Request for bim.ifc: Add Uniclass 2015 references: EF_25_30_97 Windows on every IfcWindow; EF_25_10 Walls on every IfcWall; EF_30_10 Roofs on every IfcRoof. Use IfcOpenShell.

First a look at what the model holds.

```python
import ifcopenshell

model = ifcopenshell.open("bim.ifc")
print(model.schema)
print("classifications:", [c.Name for c in model.by_type("IfcClassification")])
for ifc_class in ("IfcDoor", "IfcRoof", "IfcStair", "IfcWall", "IfcWindow"):
    print(ifc_class, len(model.by_type(ifc_class)))
```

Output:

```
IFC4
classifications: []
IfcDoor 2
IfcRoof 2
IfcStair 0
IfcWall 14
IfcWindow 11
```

```python
import ifcopenshell
import ifcopenshell.api.classification

model = ifcopenshell.open("bim.ifc")

system = ifcopenshell.api.classification.add_classification(model, classification="Uniclass 2015")

codes = {
    "IfcWindow": ("EF_25_30_97", "Windows"),
    "IfcWall": ("EF_25_10", "Walls"),
    "IfcRoof": ("EF_30_10", "Roofs"),
}
for ifc_class, (code, name) in codes.items():
    products = model.by_type(ifc_class)
    ifcopenshell.api.classification.add_reference(
        model, products=products, classification=system, identification=code, name=name
    )
    print(code, len(products))

model.write("bim_updated.ifc")
```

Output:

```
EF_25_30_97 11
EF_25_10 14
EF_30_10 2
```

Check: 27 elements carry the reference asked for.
